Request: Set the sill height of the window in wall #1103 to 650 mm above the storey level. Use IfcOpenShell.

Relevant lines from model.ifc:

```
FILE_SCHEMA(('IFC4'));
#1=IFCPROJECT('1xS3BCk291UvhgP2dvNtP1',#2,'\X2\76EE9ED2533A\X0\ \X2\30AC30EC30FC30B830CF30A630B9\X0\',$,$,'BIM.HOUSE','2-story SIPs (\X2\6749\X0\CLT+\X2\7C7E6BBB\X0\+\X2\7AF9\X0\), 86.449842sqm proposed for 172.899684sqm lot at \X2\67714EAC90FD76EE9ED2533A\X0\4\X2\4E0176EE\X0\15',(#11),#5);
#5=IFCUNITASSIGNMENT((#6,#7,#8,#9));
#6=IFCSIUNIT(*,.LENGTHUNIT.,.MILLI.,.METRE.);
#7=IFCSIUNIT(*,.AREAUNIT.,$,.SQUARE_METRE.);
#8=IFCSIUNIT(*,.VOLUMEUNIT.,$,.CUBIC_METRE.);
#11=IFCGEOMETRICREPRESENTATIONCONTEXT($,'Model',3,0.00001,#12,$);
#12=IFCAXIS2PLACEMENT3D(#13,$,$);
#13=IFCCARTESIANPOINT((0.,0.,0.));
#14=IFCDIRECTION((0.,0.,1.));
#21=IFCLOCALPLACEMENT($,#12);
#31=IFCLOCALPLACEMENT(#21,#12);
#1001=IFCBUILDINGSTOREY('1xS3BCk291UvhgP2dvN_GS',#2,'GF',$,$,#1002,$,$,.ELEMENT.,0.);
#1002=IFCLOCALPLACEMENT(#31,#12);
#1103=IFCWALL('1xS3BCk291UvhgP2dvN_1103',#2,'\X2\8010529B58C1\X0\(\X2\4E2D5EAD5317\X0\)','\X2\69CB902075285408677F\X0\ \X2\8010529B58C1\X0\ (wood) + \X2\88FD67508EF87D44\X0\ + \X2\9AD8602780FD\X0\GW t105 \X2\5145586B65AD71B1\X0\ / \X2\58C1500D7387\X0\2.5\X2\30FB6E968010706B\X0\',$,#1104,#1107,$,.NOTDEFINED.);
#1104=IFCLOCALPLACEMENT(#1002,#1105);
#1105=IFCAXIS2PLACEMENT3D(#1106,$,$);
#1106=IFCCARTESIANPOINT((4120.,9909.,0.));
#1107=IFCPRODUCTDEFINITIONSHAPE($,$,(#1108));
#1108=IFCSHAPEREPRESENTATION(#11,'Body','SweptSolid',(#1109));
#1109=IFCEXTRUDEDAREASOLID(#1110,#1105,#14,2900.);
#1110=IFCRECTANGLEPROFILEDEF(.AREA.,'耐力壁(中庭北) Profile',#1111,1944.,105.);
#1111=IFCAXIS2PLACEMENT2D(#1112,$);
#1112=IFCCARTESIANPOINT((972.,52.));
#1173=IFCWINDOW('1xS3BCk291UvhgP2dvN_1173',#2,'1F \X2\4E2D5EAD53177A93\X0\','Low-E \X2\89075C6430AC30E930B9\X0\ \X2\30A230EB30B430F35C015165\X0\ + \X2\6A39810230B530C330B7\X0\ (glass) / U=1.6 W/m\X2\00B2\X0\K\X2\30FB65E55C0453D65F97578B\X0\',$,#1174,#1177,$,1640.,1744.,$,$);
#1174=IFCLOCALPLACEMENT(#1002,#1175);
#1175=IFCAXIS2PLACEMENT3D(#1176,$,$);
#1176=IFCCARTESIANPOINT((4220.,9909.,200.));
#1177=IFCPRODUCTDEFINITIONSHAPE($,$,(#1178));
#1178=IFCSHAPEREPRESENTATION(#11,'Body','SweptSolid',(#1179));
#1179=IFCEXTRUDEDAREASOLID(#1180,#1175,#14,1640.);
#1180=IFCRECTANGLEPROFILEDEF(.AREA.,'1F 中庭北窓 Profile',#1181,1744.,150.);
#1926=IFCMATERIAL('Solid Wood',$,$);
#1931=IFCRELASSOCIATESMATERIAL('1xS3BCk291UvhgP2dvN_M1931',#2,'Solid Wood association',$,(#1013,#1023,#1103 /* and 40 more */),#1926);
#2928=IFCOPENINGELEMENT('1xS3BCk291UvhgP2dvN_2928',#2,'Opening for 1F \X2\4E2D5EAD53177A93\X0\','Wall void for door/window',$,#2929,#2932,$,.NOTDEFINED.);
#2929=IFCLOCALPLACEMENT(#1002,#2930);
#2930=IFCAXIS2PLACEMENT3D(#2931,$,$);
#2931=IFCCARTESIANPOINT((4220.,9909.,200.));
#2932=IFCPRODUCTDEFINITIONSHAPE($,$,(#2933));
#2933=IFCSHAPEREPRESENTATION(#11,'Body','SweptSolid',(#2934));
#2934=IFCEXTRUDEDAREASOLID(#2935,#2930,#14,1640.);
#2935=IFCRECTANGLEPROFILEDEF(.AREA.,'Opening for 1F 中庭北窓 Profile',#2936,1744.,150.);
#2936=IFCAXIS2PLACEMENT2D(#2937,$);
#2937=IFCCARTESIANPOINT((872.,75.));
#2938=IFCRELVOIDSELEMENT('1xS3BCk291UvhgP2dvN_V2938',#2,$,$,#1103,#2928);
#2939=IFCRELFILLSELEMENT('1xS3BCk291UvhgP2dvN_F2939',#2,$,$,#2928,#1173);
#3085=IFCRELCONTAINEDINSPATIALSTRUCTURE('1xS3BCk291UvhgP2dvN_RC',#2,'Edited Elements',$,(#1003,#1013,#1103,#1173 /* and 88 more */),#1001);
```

```python
import numpy as np
import ifcopenshell
import ifcopenshell.api.geometry
import ifcopenshell.geom
import ifcopenshell.util.element
import ifcopenshell.util.placement
import ifcopenshell.util.shape
import ifcopenshell.util.unit

model = ifcopenshell.open("model.ifc")
unit_scale = ifcopenshell.util.unit.calculate_unit_scale(model)

window = model.by_guid("1xS3BCk291UvhgP2dvN_1173")
opening = window.FillsVoids[0].RelatingOpeningElement
storey = ifcopenshell.util.element.get_container(window, ifc_class="IfcBuildingStorey")
level = ifcopenshell.util.placement.get_local_placement(storey.ObjectPlacement)[2, 3]

# The opening's origin need not be at the sill, so measure its lowest point.
shape = ifcopenshell.geom.create_shape(ifcopenshell.geom.settings(), opening)
bottom = ifcopenshell.util.shape.get_shape_bottom_elevation(shape, shape.geometry) / unit_scale
dz = level + 0.65 / unit_scale - bottom

shift = np.array([0.0, 0.0, dz])
# The window is not placed relative to its opening, so move both.
for product in (opening, window):
    matrix = ifcopenshell.util.placement.get_local_placement(product.ObjectPlacement)
    matrix[:3, 3] += shift
    ifcopenshell.api.geometry.edit_object_placement(model, product=product, matrix=matrix, is_si=False)

print(f"moved by {dz * unit_scale:+.3f} m")

model.write("model_edited.ifc")
```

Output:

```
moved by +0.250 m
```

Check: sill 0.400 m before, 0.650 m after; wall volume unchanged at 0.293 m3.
